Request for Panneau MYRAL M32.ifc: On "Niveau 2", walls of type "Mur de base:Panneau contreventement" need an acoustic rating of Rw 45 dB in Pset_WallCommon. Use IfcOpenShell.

First a look at what the model holds.

```python
import ifcopenshell
import ifcopenshell.util.element

model = ifcopenshell.open("Panneau MYRAL M32.ifc")
print(model.schema)
storey = next(s for s in model.by_type("IfcBuildingStorey") if s.Name == "Niveau 2")
walls = [e for e in ifcopenshell.util.element.get_decomposition(storey) if e.is_a("IfcWall")]
seen = {}
for e in walls:
    element_type = ifcopenshell.util.element.get_type(e)
    key = (element_type.Name if element_type != e and element_type else None, ifcopenshell.util.element.get_pset(e, "Pset_WallCommon", "AcousticRating"))
    seen[key] = seen.get(key, 0) + 1
for (name, value), count in sorted(seen.items(), key=str):
    print(count, "x", name, "|", value)
```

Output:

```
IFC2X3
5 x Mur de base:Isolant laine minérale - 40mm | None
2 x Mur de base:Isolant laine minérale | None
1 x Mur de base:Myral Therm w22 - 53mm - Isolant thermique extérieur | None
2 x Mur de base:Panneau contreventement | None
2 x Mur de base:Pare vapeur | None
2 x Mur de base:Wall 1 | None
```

```python
import ifcopenshell
import ifcopenshell.api.pset
import ifcopenshell.util.element

model = ifcopenshell.open("Panneau MYRAL M32.ifc")

storey = next(s for s in model.by_type("IfcBuildingStorey") if s.Name == "Niveau 2")
walls = [e for e in ifcopenshell.util.element.get_decomposition(storey) if e.is_a("IfcWall")]

count = 0
for e in walls:
    element_type = ifcopenshell.util.element.get_type(e)
    if element_type in (None, e) or element_type.Name != "Mur de base:Panneau contreventement":
        continue
    # add_pset returns the element's existing set when there is one.
    pset = ifcopenshell.api.pset.add_pset(model, product=e, name="Pset_WallCommon")
    ifcopenshell.api.pset.edit_pset(model, pset=pset, properties={"AcousticRating": "Rw 45 dB"})
    count += 1

print(count, "walls updated")

model.write("Panneau MYRAL M32_rev.ifc")
```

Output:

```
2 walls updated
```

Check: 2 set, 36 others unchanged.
